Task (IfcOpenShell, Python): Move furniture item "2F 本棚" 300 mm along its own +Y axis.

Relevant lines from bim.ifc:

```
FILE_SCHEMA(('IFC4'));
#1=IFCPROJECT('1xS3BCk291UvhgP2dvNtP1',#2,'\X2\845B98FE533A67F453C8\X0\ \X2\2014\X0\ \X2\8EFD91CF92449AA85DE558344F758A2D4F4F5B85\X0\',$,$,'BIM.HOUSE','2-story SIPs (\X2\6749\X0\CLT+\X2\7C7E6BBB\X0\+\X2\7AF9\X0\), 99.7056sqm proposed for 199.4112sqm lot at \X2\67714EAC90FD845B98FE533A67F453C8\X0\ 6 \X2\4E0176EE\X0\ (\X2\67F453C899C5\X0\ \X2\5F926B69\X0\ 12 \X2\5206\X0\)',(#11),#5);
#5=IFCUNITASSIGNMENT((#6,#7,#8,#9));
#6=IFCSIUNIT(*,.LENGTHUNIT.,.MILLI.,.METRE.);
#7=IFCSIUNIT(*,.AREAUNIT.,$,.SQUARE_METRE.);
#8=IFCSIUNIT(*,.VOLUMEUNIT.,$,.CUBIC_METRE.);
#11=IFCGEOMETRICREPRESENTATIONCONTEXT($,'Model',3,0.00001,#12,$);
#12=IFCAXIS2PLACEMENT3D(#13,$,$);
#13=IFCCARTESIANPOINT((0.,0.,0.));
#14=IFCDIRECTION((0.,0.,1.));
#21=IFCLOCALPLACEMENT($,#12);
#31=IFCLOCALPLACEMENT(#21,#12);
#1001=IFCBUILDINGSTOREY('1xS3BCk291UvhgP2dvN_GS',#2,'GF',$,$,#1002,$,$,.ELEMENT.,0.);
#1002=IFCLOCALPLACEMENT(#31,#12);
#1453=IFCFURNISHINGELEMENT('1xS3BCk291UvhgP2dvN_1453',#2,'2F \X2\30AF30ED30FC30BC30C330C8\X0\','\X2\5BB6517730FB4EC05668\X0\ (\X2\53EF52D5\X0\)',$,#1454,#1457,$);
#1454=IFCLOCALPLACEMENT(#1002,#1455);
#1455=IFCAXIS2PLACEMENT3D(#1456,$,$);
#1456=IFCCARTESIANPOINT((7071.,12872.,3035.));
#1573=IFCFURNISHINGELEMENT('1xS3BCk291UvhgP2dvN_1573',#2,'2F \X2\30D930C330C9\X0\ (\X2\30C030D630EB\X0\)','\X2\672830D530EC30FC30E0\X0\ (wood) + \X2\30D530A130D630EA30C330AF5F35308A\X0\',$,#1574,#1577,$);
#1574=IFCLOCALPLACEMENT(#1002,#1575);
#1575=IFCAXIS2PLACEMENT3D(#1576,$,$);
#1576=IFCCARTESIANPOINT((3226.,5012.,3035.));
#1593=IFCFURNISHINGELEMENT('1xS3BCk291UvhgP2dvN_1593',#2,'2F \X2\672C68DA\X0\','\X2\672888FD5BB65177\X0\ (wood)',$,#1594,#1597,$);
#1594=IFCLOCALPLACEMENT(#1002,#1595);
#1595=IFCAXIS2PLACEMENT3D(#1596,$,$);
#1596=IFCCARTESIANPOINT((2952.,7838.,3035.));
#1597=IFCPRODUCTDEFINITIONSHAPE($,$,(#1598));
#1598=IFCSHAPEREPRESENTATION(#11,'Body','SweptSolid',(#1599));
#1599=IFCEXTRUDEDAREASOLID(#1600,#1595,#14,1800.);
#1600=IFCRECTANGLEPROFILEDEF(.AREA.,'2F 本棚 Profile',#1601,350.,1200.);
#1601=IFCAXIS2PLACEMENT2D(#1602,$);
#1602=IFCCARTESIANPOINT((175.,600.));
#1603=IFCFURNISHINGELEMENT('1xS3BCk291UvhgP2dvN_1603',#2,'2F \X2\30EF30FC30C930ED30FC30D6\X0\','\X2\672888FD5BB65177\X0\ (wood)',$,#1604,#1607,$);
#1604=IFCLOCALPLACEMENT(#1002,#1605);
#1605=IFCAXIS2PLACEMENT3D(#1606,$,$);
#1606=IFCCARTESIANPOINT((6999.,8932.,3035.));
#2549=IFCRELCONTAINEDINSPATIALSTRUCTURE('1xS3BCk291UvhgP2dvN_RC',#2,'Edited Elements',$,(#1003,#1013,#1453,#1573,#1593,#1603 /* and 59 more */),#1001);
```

```python
import ifcopenshell
import ifcopenshell.api.geometry
import ifcopenshell.util.placement
import ifcopenshell.util.unit

model = ifcopenshell.open("bim.ifc")
unit_scale = ifcopenshell.util.unit.calculate_unit_scale(model)

item = model.by_guid("1xS3BCk291UvhgP2dvN_1593")
matrix = ifcopenshell.util.placement.get_local_placement(item.ObjectPlacement)
matrix[:3, 3] += matrix[:3, 1] * 0.3 / unit_scale
ifcopenshell.api.geometry.edit_object_placement(model, product=item, matrix=matrix, is_si=False)

print(ifcopenshell.util.placement.get_local_placement(item.ObjectPlacement).round(3) + 0.0)

model.write("bim_v2.ifc")
```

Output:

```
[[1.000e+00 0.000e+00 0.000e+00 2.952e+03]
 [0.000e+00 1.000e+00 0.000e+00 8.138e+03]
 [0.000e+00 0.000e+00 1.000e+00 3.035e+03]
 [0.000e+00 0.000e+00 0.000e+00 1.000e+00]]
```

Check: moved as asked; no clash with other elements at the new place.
